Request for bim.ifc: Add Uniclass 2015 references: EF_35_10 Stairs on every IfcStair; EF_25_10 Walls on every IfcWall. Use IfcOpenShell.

First a look at what the model holds.

```python
import ifcopenshell

model = ifcopenshell.open("bim.ifc")
print(model.schema)
print("classifications:", [c.Name for c in model.by_type("IfcClassification")])
for ifc_class in ("IfcDoor", "IfcRoof", "IfcStair", "IfcWall", "IfcWindow"):
    print(ifc_class, len(model.by_type(ifc_class)))
```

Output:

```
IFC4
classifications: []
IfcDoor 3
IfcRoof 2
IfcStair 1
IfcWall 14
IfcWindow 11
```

```python
import ifcopenshell
import ifcopenshell.api.classification

model = ifcopenshell.open("bim.ifc")

system = ifcopenshell.api.classification.add_classification(model, classification="Uniclass 2015")

codes = {
    "IfcStair": ("EF_35_10", "Stairs"),
    "IfcWall": ("EF_25_10", "Walls"),
}
for ifc_class, (code, name) in codes.items():
    products = model.by_type(ifc_class)
    ifcopenshell.api.classification.add_reference(
        model, products=products, classification=system, identification=code, name=name
    )
    print(code, len(products))

model.write("bim-out.ifc")
```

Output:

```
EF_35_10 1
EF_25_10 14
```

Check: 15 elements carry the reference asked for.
